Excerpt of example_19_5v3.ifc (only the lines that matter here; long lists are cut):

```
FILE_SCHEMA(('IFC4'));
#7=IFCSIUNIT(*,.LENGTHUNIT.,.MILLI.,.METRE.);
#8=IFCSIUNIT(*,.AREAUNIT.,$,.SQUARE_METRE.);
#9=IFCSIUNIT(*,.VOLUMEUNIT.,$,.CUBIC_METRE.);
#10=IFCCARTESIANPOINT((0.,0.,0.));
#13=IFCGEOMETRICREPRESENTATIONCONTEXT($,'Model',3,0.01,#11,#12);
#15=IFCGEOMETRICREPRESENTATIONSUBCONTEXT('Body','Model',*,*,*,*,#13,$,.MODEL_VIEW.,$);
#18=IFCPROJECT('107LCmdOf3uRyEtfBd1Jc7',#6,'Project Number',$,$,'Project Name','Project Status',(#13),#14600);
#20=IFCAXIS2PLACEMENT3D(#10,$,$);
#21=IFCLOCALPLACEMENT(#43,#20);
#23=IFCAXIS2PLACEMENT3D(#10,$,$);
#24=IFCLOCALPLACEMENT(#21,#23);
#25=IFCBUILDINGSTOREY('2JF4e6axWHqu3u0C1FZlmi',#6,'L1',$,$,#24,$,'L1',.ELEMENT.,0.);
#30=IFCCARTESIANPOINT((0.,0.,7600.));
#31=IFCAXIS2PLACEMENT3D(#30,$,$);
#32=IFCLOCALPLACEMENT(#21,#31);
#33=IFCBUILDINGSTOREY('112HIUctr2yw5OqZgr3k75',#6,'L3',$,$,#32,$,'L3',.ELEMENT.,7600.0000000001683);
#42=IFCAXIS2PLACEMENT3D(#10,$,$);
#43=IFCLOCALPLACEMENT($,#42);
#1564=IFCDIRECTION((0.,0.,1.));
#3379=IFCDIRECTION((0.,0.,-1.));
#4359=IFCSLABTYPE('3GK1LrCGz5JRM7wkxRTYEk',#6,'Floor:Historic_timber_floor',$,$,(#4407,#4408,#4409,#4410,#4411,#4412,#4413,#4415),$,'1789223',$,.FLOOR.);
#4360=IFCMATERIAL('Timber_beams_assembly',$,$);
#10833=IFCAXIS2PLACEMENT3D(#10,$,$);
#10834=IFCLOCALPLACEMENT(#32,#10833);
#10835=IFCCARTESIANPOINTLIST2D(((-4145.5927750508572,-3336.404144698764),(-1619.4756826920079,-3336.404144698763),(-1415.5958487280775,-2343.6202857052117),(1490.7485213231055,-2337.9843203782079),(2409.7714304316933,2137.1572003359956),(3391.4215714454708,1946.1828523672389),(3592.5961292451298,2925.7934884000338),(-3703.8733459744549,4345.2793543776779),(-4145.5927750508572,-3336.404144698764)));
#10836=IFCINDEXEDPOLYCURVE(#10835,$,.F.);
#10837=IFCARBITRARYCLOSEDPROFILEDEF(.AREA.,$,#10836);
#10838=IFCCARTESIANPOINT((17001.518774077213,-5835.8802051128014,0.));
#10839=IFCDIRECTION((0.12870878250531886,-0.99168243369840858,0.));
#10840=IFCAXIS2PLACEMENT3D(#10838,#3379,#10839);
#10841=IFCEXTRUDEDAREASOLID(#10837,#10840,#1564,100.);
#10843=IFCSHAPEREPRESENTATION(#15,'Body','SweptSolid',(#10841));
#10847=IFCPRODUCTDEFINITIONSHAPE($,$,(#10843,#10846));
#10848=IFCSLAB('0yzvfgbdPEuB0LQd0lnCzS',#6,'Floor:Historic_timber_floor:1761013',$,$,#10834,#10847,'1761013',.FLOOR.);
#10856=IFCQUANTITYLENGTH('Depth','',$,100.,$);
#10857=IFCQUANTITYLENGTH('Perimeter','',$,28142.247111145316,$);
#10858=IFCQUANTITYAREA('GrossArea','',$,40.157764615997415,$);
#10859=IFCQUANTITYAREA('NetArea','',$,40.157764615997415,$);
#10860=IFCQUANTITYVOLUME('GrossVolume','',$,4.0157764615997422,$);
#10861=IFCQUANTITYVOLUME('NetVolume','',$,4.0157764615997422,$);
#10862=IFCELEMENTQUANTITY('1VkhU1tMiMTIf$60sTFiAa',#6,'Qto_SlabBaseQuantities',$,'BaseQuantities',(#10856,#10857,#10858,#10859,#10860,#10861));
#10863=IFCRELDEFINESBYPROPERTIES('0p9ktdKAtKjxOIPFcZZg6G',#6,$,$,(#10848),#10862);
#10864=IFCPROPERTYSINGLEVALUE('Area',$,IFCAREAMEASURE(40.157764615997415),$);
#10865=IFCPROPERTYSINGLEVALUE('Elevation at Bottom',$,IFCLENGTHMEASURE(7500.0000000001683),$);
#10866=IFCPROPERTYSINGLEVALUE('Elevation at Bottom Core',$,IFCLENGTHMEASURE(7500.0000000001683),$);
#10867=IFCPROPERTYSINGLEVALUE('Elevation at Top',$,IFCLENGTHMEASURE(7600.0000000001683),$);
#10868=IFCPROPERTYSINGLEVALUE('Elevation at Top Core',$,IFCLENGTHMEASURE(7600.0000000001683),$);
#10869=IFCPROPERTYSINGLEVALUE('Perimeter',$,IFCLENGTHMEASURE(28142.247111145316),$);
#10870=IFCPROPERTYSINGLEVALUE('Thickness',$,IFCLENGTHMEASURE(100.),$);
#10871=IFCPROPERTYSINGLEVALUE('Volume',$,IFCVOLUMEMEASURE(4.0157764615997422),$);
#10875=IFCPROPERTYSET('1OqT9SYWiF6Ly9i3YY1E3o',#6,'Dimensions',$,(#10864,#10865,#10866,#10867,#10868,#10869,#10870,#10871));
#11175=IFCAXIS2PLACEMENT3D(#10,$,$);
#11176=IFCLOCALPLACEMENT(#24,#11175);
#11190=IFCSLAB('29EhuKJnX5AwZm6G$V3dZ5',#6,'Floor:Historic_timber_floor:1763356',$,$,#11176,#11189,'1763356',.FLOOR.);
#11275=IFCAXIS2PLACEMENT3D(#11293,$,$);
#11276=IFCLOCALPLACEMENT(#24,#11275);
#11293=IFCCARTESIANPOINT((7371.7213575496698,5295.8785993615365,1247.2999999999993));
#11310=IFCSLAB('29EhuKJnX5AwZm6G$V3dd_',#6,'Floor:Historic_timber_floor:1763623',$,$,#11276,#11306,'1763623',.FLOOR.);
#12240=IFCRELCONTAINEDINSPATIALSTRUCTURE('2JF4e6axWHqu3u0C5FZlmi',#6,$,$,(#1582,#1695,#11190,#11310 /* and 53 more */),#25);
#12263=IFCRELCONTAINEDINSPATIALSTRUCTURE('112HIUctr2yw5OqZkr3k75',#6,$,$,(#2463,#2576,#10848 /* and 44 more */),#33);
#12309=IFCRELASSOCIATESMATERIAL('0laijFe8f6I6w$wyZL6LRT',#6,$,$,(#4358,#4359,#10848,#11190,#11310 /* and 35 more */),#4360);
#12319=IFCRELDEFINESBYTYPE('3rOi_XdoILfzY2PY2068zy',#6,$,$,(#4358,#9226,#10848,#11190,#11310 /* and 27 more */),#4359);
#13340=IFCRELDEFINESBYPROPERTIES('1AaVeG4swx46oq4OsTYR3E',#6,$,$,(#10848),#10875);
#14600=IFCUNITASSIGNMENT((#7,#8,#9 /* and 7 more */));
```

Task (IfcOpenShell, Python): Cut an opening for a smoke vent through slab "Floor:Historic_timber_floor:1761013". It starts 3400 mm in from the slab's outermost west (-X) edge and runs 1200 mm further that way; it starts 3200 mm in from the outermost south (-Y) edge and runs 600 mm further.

```python
import numpy as np
import ifcopenshell
import ifcopenshell.api.feature
import ifcopenshell.api.geometry
import ifcopenshell.api.pset
import ifcopenshell.api.root
import ifcopenshell.geom
import ifcopenshell.util.element
import ifcopenshell.util.placement
import ifcopenshell.util.representation
import ifcopenshell.util.shape
import ifcopenshell.util.unit

model = ifcopenshell.open("example_19_5v3.ifc")
unit_scale = ifcopenshell.util.unit.calculate_unit_scale(model)
area_scale = ifcopenshell.util.unit.calculate_unit_scale(model, "AREAUNIT")
volume_scale = ifcopenshell.util.unit.calculate_unit_scale(model, "VOLUMEUNIT")
settings = ifcopenshell.geom.settings()


def volume(element):
    """Net volume in cubic metres, openings subtracted."""
    shape = ifcopenshell.geom.create_shape(settings, element)
    return ifcopenshell.util.shape.get_volume(shape.geometry)


slab = model.by_guid("0yzvfgbdPEuB0LQd0lnCzS")
before = volume(slab)

# Extent in the slab's own axes, in metres. The edges named are its -X and -Y sides.
slab_shape = ifcopenshell.geom.create_shape(settings, slab)
vertices = ifcopenshell.util.shape.get_vertices(slab_shape.geometry)
x_min, y_min, bottom = vertices.min(axis=0)
top = vertices[:, 2].max()

opening = ifcopenshell.api.root.create_entity(model, ifc_class="IfcOpeningElement", name="Smoke vent opening", predefined_type="OPENING")
context = ifcopenshell.util.representation.get_context(model, "Model", "Body", "MODEL_VIEW")
width, depth = 1.2, 0.6
outline = [(0.0, 0.0), (width, 0.0), (width, depth), (0.0, depth), (0.0, 0.0)]
# Overshoot both faces by 50 mm so the cut is clean.
shape = ifcopenshell.api.geometry.add_slab_representation(
    model, context=context, depth=top - bottom + 0.1, polyline=outline
)
ifcopenshell.api.geometry.assign_representation(model, product=opening, representation=shape)

matrix = ifcopenshell.util.placement.get_local_placement(slab.ObjectPlacement)
matrix[:, 3] = matrix @ np.append(np.array([x_min + 3.4, y_min + 3.2, bottom - 0.05]) / unit_scale, 1.0)
ifcopenshell.api.geometry.edit_object_placement(model, product=opening, matrix=matrix, is_si=False)
ifcopenshell.api.feature.add_feature(model, feature=opening, element=slab)

after = volume(slab)

# Update the slab's stored quantities.
qto = model.by_id(ifcopenshell.util.element.get_pset(slab, "Qto_SlabBaseQuantities", should_inherit=False)["id"])
ifcopenshell.api.pset.edit_qto(model, qto=qto, properties={
    "NetArea": after / (top - bottom) / area_scale,
    "NetVolume": after / volume_scale,
})
pset = model.by_id(ifcopenshell.util.element.get_pset(slab, "Dimensions", should_inherit=False)["id"])
ifcopenshell.api.pset.edit_pset(model, pset=pset, properties={
    "Area": model.create_entity("IfcAreaMeasure", after / (top - bottom) / area_scale),
    "Volume": model.create_entity("IfcVolumeMeasure", after / volume_scale),
})

print(f"slab volume {before:.3f} -> {after:.3f} m3")

model.write("example_19_5v3_rev.ifc")
```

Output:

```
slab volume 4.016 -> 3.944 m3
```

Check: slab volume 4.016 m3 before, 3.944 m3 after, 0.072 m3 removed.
